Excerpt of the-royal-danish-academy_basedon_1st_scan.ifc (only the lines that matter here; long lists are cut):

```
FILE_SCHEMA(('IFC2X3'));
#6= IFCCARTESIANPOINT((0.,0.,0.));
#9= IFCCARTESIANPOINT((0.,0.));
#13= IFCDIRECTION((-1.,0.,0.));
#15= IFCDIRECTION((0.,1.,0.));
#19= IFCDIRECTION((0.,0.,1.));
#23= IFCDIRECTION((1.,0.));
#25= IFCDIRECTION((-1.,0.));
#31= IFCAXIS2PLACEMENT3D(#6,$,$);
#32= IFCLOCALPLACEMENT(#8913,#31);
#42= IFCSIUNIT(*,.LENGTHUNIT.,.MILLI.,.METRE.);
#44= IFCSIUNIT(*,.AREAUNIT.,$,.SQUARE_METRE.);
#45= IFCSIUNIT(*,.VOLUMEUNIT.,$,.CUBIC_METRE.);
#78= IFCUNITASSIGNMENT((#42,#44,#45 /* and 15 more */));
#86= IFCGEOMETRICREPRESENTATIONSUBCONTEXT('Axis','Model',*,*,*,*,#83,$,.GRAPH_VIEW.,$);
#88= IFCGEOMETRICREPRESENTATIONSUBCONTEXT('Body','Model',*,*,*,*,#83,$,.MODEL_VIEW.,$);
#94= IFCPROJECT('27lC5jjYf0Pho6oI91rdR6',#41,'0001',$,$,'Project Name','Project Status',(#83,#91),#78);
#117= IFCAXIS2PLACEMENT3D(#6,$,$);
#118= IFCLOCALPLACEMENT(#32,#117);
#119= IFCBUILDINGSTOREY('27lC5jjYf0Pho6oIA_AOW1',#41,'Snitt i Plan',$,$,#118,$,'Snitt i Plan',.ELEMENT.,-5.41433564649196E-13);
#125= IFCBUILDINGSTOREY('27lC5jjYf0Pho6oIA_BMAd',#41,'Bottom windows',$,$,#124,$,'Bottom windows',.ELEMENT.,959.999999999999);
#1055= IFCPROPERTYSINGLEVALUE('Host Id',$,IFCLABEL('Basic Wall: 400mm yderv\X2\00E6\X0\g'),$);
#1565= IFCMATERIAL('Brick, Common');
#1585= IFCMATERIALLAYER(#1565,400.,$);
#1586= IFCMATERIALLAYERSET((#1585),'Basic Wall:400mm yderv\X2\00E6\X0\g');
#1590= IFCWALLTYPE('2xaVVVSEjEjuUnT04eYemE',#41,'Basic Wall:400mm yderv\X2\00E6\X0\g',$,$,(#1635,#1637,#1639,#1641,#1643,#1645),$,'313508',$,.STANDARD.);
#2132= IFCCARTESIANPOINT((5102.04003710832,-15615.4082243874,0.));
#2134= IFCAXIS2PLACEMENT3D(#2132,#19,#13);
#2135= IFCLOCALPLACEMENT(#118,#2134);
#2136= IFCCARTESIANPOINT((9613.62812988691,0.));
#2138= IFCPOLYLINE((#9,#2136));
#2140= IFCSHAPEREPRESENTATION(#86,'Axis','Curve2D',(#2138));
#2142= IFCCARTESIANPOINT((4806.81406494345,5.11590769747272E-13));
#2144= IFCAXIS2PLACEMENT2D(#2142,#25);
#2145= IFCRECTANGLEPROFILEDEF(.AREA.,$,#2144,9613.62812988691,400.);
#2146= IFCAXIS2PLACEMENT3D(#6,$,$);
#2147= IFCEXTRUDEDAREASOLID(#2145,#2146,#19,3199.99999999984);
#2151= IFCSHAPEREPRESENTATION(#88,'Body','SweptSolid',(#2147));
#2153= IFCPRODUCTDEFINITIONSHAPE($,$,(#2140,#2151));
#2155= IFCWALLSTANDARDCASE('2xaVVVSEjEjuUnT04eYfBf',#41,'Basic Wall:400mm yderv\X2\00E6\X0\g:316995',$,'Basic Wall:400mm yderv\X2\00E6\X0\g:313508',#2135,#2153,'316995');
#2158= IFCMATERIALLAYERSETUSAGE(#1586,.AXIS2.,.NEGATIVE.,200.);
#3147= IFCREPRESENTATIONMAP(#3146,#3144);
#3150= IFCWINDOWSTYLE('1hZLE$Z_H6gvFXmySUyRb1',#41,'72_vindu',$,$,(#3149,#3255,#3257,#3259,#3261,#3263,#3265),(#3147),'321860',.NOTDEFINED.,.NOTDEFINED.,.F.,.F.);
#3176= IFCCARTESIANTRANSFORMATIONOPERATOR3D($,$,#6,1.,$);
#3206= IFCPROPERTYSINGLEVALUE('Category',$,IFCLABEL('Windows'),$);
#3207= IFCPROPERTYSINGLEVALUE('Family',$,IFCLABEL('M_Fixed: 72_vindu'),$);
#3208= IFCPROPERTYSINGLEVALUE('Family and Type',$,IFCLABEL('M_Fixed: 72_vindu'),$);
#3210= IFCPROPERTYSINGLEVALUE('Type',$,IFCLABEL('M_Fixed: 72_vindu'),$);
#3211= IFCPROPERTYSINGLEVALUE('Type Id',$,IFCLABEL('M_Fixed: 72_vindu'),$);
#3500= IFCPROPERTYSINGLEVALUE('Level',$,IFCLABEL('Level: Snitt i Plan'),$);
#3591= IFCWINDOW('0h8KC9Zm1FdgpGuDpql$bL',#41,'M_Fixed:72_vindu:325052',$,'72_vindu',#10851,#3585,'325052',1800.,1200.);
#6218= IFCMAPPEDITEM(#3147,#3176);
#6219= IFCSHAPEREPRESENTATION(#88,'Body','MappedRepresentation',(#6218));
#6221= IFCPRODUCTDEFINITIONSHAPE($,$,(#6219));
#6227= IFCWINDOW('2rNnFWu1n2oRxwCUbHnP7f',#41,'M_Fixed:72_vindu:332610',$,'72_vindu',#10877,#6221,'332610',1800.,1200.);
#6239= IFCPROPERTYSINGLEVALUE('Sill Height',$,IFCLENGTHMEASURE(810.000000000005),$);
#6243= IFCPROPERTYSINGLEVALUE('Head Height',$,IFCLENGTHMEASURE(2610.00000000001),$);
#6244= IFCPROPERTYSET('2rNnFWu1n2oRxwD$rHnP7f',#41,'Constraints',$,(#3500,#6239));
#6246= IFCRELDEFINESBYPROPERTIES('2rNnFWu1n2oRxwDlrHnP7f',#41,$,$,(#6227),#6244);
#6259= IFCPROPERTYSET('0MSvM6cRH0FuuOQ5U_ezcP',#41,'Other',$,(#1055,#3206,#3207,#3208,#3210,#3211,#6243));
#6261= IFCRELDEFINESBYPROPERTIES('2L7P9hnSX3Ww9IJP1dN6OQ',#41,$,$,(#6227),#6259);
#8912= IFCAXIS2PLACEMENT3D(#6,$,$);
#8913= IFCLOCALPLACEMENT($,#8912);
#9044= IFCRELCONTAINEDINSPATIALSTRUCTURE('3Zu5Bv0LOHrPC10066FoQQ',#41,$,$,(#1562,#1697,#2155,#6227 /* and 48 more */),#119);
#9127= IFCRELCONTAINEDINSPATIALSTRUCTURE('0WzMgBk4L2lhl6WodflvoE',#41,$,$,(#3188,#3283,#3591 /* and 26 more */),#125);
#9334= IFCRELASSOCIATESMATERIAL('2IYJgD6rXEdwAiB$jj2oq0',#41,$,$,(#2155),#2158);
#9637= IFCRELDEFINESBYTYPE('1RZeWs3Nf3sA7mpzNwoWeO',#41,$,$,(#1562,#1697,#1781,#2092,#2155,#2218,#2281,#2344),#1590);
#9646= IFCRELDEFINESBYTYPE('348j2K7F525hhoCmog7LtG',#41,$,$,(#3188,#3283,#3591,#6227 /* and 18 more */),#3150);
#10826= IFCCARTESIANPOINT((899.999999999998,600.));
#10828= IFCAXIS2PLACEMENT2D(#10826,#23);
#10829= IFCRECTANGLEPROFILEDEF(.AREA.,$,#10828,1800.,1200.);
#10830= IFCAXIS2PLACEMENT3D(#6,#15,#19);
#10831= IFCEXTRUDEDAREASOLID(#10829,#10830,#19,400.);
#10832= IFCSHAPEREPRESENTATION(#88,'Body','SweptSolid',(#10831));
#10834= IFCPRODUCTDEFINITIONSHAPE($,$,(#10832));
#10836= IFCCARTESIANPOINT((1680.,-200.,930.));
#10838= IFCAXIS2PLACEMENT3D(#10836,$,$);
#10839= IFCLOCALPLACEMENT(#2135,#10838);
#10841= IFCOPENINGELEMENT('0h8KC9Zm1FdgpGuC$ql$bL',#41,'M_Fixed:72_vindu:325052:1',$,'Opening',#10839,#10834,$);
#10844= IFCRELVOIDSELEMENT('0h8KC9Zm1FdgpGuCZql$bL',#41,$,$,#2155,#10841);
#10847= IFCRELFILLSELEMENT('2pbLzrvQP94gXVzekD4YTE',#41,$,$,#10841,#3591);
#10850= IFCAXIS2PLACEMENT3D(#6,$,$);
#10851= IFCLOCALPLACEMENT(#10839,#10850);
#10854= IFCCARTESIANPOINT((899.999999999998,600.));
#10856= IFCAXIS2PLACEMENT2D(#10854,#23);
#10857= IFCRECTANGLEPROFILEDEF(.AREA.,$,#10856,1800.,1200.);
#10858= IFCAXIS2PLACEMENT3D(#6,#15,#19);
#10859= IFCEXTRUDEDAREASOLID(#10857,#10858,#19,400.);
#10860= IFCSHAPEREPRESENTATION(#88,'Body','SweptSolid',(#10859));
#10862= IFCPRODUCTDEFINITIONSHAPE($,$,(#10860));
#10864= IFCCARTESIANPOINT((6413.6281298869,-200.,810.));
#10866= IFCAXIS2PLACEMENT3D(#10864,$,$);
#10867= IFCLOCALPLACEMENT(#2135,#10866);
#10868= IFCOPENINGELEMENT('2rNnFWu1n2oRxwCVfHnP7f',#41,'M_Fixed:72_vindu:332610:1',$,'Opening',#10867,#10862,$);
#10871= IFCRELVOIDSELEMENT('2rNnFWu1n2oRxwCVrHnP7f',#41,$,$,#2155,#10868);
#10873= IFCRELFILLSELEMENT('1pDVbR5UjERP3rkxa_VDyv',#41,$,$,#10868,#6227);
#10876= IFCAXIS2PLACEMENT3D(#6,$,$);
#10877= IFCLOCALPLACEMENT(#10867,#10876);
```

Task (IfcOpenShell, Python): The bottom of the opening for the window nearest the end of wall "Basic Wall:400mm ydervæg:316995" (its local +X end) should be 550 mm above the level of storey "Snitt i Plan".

```python
import numpy as np
import ifcopenshell
import ifcopenshell.api.geometry
import ifcopenshell.api.pset
import ifcopenshell.geom
import ifcopenshell.util.element
import ifcopenshell.util.placement
import ifcopenshell.util.shape
import ifcopenshell.util.unit

model = ifcopenshell.open("the-royal-danish-academy_basedon_1st_scan.ifc")
unit_scale = ifcopenshell.util.unit.calculate_unit_scale(model)

window = model.by_id(6227)
opening = window.FillsVoids[0].RelatingOpeningElement
storey = ifcopenshell.util.element.get_container(window, ifc_class="IfcBuildingStorey")
level = ifcopenshell.util.placement.get_local_placement(storey.ObjectPlacement)[2, 3]

# The opening's origin need not be at the sill, so measure its lowest point.
shape = ifcopenshell.geom.create_shape(ifcopenshell.geom.settings(), opening)
bottom = ifcopenshell.util.shape.get_shape_bottom_elevation(shape, shape.geometry) / unit_scale
dz = level + 550.0 - bottom

shift = np.array([0.0, 0.0, dz])
# The window is placed relative to its opening, so it follows when the opening moves.
matrix = ifcopenshell.util.placement.get_local_placement(opening.ObjectPlacement)
matrix[:3, 3] += shift
ifcopenshell.api.geometry.edit_object_placement(
    model, product=opening, matrix=matrix, is_si=False, should_transform_children=True
)

# Keep the stored heights in step.
pset = model.by_id(ifcopenshell.util.element.get_pset(window, "Constraints", should_inherit=False)["id"])
ifcopenshell.api.pset.edit_pset(model, pset=pset, properties={
    "Sill Height": model.create_entity("IfcLengthMeasure", ifcopenshell.util.element.get_pset(window, "Constraints", "Sill Height") + dz),
})
pset = model.by_id(ifcopenshell.util.element.get_pset(window, "Other", should_inherit=False)["id"])
ifcopenshell.api.pset.edit_pset(model, pset=pset, properties={
    "Head Height": model.create_entity("IfcLengthMeasure", ifcopenshell.util.element.get_pset(window, "Other", "Head Height") + dz),
})

print(f"moved by {dz * unit_scale:+.3f} m")

model.write("the-royal-danish-academy_basedon_1st_scan_updated.ifc")
```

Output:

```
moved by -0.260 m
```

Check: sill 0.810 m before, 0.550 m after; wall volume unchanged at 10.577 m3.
